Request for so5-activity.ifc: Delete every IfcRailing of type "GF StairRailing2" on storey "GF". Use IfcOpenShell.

First a look at what the model holds.

```python
import ifcopenshell
import ifcopenshell.util.element

model = ifcopenshell.open("so5-activity.ifc")
print(model.schema)
storey = next(s for s in model.by_type("IfcBuildingStorey") if s.Name == "GF")
railings = [e for e in ifcopenshell.util.element.get_decomposition(storey) if e.is_a("IfcRailing")]
seen = {}
for e in railings:
    element_type = ifcopenshell.util.element.get_type(e)
    name = element_type.Name if element_type not in (None, e) else None
    seen[name] = seen.get(name, 0) + 1
for name, count in sorted(seen.items(), key=str):
    print(count, "x", name)
```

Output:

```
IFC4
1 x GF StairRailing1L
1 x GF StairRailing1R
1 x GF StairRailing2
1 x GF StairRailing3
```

```python
import ifcopenshell
import ifcopenshell.api.root
import ifcopenshell.util.element

model = ifcopenshell.open("so5-activity.ifc")

storey = next(s for s in model.by_type("IfcBuildingStorey") if s.Name == "GF")
railings = [e for e in ifcopenshell.util.element.get_decomposition(storey) if e.is_a("IfcRailing")]
targets = [e for e in railings if (t := ifcopenshell.util.element.get_type(e)) not in (None, e) and t.Name == "GF StairRailing2"]

for e in targets:
    ifcopenshell.api.root.remove_product(model, product=e)
print(len(targets), "removed")

model.write("so5-activity_updated.ifc")
```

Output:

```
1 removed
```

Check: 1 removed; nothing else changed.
